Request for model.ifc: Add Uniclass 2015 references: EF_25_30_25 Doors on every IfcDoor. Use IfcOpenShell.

First a look at what the model holds.

```python
import ifcopenshell

model = ifcopenshell.open("model.ifc")
print(model.schema)
print("classifications:", [c.Name for c in model.by_type("IfcClassification")])
for ifc_class in ("IfcDoor", "IfcRoof", "IfcStair", "IfcWall", "IfcWindow"):
    print(ifc_class, len(model.by_type(ifc_class)))
```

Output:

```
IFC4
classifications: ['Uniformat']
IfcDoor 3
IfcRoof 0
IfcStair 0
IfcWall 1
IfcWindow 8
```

```python
import ifcopenshell
import ifcopenshell.api.classification

model = ifcopenshell.open("model.ifc")

system = ifcopenshell.api.classification.add_classification(model, classification="Uniclass 2015")

codes = {
    "IfcDoor": ("EF_25_30_25", "Doors"),
}
for ifc_class, (code, name) in codes.items():
    products = model.by_type(ifc_class)
    ifcopenshell.api.classification.add_reference(
        model, products=products, classification=system, identification=code, name=name
    )
    print(code, len(products))

model.write("model_edited.ifc")
```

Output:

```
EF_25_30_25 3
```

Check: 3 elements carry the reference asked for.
